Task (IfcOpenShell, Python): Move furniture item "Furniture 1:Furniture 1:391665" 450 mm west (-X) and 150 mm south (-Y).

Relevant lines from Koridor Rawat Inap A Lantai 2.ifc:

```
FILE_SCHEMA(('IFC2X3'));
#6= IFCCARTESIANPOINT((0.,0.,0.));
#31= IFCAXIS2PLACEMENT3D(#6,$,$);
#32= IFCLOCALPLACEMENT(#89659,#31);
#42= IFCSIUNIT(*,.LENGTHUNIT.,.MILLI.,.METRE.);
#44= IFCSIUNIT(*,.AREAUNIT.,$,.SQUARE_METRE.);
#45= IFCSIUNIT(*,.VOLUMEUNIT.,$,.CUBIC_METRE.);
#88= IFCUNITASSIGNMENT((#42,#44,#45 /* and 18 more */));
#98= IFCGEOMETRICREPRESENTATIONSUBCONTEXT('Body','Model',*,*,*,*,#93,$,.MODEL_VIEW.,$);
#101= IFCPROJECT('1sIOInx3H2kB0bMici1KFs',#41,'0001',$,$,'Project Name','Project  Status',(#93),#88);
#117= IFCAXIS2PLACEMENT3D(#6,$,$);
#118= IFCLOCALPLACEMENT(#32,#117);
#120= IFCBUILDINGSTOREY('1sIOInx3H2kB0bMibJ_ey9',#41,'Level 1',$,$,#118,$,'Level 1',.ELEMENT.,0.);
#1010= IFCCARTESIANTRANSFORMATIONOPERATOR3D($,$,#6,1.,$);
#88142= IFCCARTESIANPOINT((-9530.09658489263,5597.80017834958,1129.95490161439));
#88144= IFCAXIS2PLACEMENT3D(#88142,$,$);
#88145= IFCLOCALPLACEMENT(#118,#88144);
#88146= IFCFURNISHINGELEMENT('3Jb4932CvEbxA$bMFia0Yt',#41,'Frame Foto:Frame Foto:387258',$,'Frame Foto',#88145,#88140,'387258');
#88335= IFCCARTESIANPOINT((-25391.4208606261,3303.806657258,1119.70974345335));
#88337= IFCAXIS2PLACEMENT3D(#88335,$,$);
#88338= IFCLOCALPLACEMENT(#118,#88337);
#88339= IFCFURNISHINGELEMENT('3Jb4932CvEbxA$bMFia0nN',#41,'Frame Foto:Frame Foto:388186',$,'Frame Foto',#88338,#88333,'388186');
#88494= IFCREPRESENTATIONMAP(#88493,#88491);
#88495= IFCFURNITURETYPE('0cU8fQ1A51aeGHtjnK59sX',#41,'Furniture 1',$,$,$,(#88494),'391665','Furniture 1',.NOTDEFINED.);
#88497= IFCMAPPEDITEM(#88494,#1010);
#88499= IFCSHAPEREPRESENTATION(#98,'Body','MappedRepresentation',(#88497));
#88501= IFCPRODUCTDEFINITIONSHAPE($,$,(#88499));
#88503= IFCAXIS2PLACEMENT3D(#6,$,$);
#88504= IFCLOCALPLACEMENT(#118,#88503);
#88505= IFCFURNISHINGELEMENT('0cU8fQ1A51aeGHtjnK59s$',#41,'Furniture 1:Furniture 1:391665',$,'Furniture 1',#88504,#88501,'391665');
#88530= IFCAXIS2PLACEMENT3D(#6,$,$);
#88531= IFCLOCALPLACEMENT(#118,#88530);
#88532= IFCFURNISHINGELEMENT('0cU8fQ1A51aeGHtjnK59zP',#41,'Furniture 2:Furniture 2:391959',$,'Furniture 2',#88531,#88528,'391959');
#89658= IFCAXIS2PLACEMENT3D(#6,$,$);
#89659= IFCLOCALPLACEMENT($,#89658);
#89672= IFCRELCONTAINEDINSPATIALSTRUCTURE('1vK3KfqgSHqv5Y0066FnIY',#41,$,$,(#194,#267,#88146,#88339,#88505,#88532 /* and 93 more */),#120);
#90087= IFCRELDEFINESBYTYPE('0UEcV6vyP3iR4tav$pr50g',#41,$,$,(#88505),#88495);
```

```python
import ifcopenshell
import ifcopenshell.api.geometry
import ifcopenshell.util.placement
import ifcopenshell.util.unit

model = ifcopenshell.open("Koridor Rawat Inap A Lantai 2.ifc")
unit_scale = ifcopenshell.util.unit.calculate_unit_scale(model)

item = model.by_guid("0cU8fQ1A51aeGHtjnK59s$")
matrix = ifcopenshell.util.placement.get_local_placement(item.ObjectPlacement)
matrix[0, 3] -= 0.45 / unit_scale
matrix[1, 3] -= 0.15 / unit_scale
ifcopenshell.api.geometry.edit_object_placement(model, product=item, matrix=matrix, is_si=False)

print(ifcopenshell.util.placement.get_local_placement(item.ObjectPlacement).round(3) + 0.0)

model.write("Koridor Rawat Inap A Lantai 2_edited.ifc")
```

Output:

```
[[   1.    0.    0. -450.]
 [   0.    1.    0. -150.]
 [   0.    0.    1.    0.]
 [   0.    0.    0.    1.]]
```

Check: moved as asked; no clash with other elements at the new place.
